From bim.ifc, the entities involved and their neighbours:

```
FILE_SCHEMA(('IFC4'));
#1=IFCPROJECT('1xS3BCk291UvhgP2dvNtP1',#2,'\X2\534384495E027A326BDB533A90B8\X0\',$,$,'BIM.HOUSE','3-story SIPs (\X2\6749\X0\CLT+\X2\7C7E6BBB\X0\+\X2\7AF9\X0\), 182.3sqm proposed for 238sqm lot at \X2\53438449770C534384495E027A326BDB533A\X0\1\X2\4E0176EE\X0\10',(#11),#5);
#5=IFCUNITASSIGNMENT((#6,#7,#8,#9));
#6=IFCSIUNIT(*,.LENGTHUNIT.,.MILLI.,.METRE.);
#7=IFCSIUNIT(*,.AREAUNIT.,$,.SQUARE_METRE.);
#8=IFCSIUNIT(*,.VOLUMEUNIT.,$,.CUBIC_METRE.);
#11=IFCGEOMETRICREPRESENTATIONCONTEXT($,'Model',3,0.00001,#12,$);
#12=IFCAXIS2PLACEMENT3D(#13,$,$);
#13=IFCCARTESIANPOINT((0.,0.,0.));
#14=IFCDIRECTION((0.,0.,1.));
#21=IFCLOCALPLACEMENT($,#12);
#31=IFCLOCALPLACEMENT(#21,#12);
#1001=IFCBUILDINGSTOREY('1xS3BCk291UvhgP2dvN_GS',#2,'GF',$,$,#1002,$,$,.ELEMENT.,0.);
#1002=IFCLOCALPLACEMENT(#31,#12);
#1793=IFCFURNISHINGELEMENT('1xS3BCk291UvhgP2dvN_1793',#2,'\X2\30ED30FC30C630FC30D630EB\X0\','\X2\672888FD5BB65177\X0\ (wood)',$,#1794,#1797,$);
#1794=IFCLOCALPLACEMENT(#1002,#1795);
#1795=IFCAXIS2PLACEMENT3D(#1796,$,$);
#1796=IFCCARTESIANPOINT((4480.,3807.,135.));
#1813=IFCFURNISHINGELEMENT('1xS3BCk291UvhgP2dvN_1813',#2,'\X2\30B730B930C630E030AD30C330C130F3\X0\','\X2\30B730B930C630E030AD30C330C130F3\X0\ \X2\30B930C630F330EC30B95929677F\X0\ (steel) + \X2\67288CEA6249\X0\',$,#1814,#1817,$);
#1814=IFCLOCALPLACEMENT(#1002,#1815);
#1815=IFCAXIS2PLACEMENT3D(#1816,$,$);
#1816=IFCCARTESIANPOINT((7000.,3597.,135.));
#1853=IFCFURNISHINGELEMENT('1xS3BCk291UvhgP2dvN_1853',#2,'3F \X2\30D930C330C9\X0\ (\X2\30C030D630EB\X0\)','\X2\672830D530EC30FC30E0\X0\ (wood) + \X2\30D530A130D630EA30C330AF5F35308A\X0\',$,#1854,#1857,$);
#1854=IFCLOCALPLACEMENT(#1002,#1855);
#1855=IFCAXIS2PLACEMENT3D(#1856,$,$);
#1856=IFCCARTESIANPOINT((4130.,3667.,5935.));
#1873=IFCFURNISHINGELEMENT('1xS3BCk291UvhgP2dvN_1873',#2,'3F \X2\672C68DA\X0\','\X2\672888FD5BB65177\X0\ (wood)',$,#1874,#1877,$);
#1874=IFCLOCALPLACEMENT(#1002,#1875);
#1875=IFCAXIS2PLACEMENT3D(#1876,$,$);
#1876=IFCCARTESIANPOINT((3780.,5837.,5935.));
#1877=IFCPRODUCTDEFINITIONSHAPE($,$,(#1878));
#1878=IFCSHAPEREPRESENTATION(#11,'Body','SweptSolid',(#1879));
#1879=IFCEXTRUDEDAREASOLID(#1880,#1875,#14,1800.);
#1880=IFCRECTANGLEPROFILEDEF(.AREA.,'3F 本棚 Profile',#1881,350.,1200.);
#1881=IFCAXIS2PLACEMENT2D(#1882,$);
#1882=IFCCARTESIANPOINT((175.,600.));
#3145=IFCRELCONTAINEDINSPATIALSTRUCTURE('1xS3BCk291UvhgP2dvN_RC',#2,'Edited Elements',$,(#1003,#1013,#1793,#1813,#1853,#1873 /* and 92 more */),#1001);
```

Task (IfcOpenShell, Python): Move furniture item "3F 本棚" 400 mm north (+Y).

```python
import ifcopenshell
import ifcopenshell.api.geometry
import ifcopenshell.util.placement

model = ifcopenshell.open("bim.ifc")

item = model.by_guid("1xS3BCk291UvhgP2dvN_1873")
matrix = ifcopenshell.util.placement.get_local_placement(item.ObjectPlacement)
matrix[1, 3] += 400.0
ifcopenshell.api.geometry.edit_object_placement(model, product=item, matrix=matrix, is_si=False)

print(ifcopenshell.util.placement.get_local_placement(item.ObjectPlacement).round(3) + 0.0)

model.write("bim_rev.ifc")
```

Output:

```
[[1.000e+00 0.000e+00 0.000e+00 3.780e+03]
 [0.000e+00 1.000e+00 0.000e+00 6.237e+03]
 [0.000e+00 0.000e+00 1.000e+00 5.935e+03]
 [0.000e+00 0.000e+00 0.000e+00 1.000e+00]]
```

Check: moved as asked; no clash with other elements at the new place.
